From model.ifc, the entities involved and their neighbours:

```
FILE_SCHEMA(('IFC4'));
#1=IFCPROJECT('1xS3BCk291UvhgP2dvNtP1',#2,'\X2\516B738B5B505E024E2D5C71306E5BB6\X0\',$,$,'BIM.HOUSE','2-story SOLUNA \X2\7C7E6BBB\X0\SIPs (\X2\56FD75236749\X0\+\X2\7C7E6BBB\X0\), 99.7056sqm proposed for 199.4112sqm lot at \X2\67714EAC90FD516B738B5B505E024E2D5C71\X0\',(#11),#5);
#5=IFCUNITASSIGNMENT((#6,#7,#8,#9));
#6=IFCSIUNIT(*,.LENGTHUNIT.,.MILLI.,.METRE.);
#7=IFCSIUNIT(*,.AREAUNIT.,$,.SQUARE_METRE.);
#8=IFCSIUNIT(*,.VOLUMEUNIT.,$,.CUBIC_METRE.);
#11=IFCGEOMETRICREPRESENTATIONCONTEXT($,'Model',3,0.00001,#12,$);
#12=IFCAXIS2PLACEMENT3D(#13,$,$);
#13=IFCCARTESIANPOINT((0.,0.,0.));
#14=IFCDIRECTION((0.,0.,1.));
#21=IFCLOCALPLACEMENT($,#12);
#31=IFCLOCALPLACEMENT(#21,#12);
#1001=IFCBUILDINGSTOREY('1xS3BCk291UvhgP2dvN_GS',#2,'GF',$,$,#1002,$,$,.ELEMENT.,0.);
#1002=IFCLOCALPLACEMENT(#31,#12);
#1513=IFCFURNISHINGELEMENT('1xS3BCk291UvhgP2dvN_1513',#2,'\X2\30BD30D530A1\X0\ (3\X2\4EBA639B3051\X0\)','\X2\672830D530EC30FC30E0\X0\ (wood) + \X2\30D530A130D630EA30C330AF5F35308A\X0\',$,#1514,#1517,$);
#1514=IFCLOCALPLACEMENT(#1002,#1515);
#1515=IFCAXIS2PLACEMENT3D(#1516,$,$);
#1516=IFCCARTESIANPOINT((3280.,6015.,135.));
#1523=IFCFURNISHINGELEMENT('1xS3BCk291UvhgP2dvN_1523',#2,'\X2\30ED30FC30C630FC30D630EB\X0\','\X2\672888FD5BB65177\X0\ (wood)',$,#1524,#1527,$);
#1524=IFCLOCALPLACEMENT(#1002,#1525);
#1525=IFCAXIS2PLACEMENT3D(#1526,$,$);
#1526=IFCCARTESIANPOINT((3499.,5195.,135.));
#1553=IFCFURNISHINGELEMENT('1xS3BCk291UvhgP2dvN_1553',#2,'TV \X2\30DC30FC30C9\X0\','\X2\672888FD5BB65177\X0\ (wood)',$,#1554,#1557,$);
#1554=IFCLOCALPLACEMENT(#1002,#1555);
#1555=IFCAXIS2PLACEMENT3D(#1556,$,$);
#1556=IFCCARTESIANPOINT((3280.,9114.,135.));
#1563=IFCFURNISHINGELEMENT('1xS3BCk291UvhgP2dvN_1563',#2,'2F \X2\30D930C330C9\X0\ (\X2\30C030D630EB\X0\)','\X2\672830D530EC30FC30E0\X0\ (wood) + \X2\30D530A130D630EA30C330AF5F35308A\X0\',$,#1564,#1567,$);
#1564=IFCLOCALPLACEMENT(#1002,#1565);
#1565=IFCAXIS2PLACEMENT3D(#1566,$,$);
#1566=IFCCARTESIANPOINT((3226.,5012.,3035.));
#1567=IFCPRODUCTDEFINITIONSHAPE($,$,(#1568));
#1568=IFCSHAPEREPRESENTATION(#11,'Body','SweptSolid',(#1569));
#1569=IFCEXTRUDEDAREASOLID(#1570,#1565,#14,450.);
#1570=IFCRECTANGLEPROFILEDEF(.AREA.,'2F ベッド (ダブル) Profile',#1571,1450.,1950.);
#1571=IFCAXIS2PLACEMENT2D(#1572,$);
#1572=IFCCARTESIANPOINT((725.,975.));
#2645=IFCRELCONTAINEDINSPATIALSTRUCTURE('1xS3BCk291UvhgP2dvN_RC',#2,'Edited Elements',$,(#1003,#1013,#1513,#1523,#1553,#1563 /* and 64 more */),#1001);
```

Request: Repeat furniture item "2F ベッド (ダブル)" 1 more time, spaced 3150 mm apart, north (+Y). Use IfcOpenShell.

```python
import numpy as np
import ifcopenshell
import ifcopenshell.api.geometry
import ifcopenshell.api.root
import ifcopenshell.util.element
import ifcopenshell.util.placement

model = ifcopenshell.open("model.ifc")


def reuse_history(source, copy):
    """copy_class also copies each property set's owner history, people and application; keep the originals."""
    for rel in copy.IsDefinedBy:
        if rel.is_a("IfcRelDefinesByProperties") and (history := rel.RelatingPropertyDefinition.OwnerHistory):
            rel.RelatingPropertyDefinition.OwnerHistory = source.OwnerHistory
            ifcopenshell.util.element.remove_deep2(model, history)


source = model.by_guid("1xS3BCk291UvhgP2dvN_1563")
base = ifcopenshell.util.placement.get_local_placement(source.ObjectPlacement)
step = np.array([0.0, 1.0, 0.0]) * 3150.0

for i in range(1, 2):
    copy = ifcopenshell.api.root.copy_class(model, product=source)
    copy.Representation = ifcopenshell.util.element.copy_deep(
        model, source.Representation, exclude=["IfcGeometricRepresentationContext", "IfcRepresentationMap"]
    )
    reuse_history(source, copy)
    matrix = base.copy()
    matrix[:3, 3] += i * step
    print("added at", matrix[:3, 3].round(3) + 0.0)
    ifcopenshell.api.geometry.edit_object_placement(model, product=copy, matrix=matrix, is_si=False)

model.write("model_updated.ifc")
```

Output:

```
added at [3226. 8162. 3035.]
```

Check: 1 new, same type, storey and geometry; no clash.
